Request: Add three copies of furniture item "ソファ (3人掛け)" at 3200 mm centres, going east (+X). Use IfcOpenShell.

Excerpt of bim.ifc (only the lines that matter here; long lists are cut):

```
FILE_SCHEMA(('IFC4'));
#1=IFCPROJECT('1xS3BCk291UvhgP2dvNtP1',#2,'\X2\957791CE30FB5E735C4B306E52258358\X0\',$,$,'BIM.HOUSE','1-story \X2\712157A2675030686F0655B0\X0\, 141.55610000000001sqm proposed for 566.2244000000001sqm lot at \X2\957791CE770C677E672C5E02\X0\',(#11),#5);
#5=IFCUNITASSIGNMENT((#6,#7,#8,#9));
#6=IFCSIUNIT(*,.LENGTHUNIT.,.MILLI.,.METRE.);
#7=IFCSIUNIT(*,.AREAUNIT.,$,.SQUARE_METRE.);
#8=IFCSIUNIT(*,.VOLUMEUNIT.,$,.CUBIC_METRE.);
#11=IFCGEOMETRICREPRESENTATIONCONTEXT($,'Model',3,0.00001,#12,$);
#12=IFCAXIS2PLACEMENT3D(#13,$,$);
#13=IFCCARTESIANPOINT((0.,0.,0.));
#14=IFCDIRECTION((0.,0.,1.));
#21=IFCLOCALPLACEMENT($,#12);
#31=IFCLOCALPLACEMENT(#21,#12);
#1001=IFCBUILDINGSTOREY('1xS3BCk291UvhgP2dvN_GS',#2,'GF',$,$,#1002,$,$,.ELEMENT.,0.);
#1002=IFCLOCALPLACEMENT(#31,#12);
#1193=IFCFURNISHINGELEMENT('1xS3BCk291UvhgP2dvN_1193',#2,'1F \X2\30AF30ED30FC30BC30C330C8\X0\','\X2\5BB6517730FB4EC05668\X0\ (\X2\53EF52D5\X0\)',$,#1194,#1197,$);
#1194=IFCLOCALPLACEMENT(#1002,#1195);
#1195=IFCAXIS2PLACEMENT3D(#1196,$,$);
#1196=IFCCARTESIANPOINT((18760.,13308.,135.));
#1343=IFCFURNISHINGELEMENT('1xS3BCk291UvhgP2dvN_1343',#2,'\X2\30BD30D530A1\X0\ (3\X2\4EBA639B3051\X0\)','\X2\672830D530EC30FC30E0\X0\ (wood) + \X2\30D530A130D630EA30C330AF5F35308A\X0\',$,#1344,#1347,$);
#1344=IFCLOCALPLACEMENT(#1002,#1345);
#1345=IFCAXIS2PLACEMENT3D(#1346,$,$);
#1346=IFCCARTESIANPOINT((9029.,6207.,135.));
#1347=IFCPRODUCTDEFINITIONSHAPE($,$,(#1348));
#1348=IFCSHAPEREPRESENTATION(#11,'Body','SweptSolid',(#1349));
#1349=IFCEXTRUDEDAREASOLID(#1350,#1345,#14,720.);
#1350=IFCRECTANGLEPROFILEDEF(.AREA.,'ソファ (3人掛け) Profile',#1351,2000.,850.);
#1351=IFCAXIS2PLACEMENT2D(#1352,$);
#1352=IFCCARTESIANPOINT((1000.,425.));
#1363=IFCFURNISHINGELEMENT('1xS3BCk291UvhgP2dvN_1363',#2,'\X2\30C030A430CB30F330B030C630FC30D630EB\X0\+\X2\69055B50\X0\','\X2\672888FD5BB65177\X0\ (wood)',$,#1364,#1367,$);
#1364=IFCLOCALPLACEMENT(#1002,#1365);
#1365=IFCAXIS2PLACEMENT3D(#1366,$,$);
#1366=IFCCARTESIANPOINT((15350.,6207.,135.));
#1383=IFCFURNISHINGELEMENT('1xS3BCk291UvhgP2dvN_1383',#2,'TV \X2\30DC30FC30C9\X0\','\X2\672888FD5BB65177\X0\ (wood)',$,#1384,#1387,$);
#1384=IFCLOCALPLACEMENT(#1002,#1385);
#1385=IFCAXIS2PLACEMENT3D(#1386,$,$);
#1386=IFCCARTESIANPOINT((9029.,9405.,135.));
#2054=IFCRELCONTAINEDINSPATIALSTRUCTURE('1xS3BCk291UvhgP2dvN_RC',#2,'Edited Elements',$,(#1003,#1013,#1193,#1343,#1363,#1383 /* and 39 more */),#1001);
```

```python
import numpy as np
import ifcopenshell
import ifcopenshell.api.geometry
import ifcopenshell.api.root
import ifcopenshell.util.element
import ifcopenshell.util.placement
import ifcopenshell.util.unit

model = ifcopenshell.open("bim.ifc")
unit_scale = ifcopenshell.util.unit.calculate_unit_scale(model)


def reuse_history(source, copy):
    """copy_class also copies each property set's owner history, people and application; keep the originals."""
    for rel in copy.IsDefinedBy:
        if rel.is_a("IfcRelDefinesByProperties") and (history := rel.RelatingPropertyDefinition.OwnerHistory):
            rel.RelatingPropertyDefinition.OwnerHistory = source.OwnerHistory
            ifcopenshell.util.element.remove_deep2(model, history)


source = model.by_guid("1xS3BCk291UvhgP2dvN_1343")
base = ifcopenshell.util.placement.get_local_placement(source.ObjectPlacement)
step = np.array([1.0, 0.0, 0.0]) * 3.2 / unit_scale

for i in range(1, 4):
    copy = ifcopenshell.api.root.copy_class(model, product=source)
    copy.Representation = ifcopenshell.util.element.copy_deep(
        model, source.Representation, exclude=["IfcGeometricRepresentationContext", "IfcRepresentationMap"]
    )
    reuse_history(source, copy)
    matrix = base.copy()
    matrix[:3, 3] += i * step
    print("added at", matrix[:3, 3].round(3) + 0.0)
    ifcopenshell.api.geometry.edit_object_placement(model, product=copy, matrix=matrix, is_si=False)

model.write("bim_edited.ifc")
```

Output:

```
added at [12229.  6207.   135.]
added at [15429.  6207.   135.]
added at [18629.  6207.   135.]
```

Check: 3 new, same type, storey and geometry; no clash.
